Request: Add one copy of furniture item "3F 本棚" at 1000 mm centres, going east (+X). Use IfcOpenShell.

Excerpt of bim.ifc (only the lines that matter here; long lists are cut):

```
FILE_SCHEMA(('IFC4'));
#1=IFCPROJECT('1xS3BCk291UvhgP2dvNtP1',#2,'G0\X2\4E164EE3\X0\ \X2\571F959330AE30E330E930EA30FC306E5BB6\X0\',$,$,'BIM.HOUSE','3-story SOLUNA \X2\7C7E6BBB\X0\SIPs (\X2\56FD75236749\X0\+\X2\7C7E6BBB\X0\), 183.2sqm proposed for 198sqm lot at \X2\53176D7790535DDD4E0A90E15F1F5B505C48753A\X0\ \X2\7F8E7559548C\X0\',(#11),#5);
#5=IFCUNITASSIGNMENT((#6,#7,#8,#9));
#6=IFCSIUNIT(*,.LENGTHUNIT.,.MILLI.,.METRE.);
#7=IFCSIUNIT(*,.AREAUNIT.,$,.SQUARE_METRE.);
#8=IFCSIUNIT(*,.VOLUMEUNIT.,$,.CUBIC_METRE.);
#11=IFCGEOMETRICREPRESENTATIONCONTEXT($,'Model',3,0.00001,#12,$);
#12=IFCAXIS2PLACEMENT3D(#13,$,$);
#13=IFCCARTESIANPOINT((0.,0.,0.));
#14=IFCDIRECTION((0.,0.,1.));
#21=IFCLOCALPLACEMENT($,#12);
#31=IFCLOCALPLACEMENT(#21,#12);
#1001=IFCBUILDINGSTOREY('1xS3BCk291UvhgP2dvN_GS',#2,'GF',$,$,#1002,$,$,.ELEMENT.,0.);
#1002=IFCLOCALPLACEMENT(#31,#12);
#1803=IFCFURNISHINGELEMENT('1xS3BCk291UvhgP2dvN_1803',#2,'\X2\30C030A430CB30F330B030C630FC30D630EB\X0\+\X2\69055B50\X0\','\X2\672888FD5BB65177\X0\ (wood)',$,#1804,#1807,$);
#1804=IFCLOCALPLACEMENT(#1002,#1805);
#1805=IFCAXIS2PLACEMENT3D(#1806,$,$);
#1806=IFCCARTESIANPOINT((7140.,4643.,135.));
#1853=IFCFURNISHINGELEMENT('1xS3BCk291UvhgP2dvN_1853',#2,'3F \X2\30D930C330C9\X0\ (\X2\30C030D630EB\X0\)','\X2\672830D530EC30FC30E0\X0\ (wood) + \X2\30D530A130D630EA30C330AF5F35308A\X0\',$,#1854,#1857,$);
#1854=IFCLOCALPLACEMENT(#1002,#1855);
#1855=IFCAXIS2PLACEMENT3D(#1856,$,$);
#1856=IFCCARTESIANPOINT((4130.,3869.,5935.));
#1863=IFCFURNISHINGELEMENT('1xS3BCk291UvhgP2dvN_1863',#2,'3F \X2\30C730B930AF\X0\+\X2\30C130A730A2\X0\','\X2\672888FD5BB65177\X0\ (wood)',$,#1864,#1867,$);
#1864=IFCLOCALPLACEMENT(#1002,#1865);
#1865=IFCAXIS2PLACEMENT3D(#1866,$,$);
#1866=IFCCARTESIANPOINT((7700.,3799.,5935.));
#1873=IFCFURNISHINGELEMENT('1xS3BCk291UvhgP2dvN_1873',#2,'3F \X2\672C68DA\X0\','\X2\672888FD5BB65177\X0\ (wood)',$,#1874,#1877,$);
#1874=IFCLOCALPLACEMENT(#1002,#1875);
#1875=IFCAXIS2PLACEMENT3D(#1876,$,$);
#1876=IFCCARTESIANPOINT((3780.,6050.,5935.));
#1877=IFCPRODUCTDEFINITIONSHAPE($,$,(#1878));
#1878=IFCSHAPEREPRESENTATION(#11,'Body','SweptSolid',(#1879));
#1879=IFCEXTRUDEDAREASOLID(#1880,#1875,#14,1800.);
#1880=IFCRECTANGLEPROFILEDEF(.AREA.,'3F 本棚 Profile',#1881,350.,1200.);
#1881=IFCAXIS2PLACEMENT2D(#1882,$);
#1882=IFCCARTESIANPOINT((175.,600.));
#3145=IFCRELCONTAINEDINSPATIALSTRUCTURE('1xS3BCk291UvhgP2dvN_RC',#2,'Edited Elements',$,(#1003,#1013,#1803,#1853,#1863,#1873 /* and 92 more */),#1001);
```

```python
import numpy as np
import ifcopenshell
import ifcopenshell.api.geometry
import ifcopenshell.api.root
import ifcopenshell.util.element
import ifcopenshell.util.placement
import ifcopenshell.util.unit

model = ifcopenshell.open("bim.ifc")
unit_scale = ifcopenshell.util.unit.calculate_unit_scale(model)


def reuse_history(source, copy):
    """copy_class also copies each property set's owner history, people and application; keep the originals."""
    for rel in copy.IsDefinedBy:
        if rel.is_a("IfcRelDefinesByProperties") and (history := rel.RelatingPropertyDefinition.OwnerHistory):
            rel.RelatingPropertyDefinition.OwnerHistory = source.OwnerHistory
            ifcopenshell.util.element.remove_deep2(model, history)


source = model.by_guid("1xS3BCk291UvhgP2dvN_1873")
base = ifcopenshell.util.placement.get_local_placement(source.ObjectPlacement)
step = np.array([1.0, 0.0, 0.0]) * 1 / unit_scale

for i in range(1, 2):
    copy = ifcopenshell.api.root.copy_class(model, product=source)
    copy.Representation = ifcopenshell.util.element.copy_deep(
        model, source.Representation, exclude=["IfcGeometricRepresentationContext", "IfcRepresentationMap"]
    )
    reuse_history(source, copy)
    matrix = base.copy()
    matrix[:3, 3] += i * step
    print("added at", matrix[:3, 3].round(3) + 0.0)
    ifcopenshell.api.geometry.edit_object_placement(model, product=copy, matrix=matrix, is_si=False)

model.write("bim-out.ifc")
```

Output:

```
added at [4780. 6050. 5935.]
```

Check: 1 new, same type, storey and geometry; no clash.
